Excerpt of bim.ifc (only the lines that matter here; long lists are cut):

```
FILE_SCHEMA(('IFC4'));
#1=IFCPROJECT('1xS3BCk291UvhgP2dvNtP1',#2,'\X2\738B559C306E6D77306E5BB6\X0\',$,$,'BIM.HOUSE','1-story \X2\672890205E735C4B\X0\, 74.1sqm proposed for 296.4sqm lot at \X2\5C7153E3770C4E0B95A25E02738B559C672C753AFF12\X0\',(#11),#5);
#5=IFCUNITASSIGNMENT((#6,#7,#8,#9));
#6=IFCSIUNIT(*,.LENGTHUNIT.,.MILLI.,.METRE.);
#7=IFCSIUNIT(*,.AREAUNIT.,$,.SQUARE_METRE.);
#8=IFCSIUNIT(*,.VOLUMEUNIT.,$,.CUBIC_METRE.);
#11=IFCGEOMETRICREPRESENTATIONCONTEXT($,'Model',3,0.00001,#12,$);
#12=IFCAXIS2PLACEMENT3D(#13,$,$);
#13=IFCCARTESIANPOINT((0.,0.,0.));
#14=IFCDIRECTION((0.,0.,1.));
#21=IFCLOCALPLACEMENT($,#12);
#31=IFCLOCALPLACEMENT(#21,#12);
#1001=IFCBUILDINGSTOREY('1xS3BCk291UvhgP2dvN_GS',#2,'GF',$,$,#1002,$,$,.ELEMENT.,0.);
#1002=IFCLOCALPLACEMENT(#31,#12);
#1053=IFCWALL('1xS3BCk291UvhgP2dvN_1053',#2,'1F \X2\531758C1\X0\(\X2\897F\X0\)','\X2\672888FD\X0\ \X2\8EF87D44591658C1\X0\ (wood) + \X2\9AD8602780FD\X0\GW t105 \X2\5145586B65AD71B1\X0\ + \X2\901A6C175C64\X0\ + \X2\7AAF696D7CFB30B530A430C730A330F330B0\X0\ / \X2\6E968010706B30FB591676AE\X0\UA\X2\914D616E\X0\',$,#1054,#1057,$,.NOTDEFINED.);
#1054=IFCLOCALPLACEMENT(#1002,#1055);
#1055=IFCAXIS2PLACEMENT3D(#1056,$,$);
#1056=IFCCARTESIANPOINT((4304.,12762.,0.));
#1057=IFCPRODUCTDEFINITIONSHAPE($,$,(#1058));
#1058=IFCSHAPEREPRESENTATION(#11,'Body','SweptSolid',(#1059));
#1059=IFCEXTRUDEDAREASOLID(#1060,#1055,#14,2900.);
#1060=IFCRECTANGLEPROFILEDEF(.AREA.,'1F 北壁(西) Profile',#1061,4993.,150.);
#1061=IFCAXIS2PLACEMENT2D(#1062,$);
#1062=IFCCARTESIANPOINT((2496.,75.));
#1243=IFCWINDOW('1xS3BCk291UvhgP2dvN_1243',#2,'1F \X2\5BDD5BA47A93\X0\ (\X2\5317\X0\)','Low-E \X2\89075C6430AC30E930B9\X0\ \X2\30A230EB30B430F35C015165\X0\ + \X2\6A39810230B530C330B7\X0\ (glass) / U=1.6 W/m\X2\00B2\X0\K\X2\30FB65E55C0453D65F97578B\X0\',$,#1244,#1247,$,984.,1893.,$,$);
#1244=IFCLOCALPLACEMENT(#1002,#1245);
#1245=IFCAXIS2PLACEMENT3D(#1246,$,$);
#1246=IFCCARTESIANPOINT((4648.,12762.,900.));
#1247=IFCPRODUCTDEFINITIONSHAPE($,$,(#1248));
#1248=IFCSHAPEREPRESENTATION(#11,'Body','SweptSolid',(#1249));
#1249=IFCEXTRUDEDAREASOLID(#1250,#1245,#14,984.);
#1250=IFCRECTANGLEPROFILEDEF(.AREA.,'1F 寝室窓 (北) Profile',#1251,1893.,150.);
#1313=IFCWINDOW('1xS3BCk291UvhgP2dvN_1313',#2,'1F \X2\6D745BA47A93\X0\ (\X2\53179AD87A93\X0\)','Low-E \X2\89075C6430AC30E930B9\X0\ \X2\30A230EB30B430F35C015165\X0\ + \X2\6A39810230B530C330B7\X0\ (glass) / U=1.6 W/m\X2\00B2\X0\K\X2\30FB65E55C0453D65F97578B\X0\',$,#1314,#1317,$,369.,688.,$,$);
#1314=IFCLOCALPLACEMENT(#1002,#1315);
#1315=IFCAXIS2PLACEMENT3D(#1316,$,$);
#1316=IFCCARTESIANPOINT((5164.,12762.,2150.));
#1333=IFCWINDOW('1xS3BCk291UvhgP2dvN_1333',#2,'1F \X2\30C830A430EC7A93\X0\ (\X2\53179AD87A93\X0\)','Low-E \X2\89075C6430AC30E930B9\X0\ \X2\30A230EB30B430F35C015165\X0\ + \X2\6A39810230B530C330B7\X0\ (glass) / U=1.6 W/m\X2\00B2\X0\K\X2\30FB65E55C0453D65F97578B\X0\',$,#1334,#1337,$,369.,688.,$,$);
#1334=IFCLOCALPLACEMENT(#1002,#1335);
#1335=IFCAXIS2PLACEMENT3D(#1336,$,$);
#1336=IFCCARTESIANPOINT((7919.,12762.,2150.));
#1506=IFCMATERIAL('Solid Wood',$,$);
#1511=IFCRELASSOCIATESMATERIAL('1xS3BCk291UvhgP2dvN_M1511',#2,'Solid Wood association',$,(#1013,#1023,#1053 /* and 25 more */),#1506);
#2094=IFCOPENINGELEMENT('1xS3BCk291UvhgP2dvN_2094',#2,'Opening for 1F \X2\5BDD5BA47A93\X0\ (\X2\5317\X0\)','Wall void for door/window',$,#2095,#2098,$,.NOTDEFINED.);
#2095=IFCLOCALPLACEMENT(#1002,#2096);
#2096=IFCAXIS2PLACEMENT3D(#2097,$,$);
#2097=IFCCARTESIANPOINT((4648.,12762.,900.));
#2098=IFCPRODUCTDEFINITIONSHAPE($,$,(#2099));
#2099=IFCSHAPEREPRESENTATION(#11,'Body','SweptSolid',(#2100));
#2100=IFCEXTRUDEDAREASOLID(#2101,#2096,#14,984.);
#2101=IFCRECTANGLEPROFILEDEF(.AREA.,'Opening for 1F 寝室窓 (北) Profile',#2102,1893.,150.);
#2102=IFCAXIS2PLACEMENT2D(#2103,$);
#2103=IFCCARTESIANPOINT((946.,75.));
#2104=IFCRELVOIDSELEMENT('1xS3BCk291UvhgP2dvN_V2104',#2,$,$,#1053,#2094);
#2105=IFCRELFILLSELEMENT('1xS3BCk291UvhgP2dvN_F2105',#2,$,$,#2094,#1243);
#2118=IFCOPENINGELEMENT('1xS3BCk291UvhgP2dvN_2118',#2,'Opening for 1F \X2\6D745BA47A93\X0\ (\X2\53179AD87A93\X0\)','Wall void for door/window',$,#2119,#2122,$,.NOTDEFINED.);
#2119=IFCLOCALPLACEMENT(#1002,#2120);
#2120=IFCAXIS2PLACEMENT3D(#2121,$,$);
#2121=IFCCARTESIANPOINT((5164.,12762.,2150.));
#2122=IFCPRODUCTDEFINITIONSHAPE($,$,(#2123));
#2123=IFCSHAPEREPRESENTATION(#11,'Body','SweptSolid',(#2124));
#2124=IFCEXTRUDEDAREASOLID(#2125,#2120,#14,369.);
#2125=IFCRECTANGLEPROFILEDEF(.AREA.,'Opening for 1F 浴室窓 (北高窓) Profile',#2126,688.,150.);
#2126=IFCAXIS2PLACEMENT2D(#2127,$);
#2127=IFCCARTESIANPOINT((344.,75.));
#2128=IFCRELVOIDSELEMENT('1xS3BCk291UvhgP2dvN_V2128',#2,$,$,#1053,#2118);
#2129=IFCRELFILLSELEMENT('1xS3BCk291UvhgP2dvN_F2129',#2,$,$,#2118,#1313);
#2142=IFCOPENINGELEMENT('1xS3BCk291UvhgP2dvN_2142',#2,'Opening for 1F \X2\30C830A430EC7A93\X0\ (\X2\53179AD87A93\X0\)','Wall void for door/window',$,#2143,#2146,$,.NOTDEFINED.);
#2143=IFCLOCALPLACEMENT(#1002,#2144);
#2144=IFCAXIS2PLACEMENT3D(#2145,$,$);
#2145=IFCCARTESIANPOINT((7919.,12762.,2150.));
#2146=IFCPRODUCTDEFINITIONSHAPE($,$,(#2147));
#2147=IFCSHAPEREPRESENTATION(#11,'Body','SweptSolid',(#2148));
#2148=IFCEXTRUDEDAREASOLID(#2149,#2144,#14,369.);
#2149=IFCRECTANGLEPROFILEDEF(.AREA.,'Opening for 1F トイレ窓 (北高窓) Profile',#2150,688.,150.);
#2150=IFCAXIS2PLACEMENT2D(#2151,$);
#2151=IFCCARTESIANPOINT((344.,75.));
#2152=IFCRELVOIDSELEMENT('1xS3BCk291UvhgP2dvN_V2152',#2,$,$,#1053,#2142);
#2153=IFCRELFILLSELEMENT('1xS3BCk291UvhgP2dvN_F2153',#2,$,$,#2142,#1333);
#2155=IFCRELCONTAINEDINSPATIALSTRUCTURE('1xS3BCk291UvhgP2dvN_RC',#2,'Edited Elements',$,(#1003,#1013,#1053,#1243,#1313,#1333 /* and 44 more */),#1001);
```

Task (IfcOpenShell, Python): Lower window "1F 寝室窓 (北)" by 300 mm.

```python
import numpy as np
import ifcopenshell
import ifcopenshell.api.geometry
import ifcopenshell.util.placement
import ifcopenshell.util.unit

model = ifcopenshell.open("bim.ifc")
unit_scale = ifcopenshell.util.unit.calculate_unit_scale(model)

window = model.by_guid("1xS3BCk291UvhgP2dvN_1243")
opening = window.FillsVoids[0].RelatingOpeningElement
dz = -300.0

shift = np.array([0.0, 0.0, dz])
# The window is not placed relative to its opening, so move both.
for product in (opening, window):
    matrix = ifcopenshell.util.placement.get_local_placement(product.ObjectPlacement)
    matrix[:3, 3] += shift
    ifcopenshell.api.geometry.edit_object_placement(model, product=product, matrix=matrix, is_si=False)

print(f"moved by {dz * unit_scale:+.3f} m")

model.write("bim_v2.ifc")
```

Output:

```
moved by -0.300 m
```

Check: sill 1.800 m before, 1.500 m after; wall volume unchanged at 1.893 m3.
